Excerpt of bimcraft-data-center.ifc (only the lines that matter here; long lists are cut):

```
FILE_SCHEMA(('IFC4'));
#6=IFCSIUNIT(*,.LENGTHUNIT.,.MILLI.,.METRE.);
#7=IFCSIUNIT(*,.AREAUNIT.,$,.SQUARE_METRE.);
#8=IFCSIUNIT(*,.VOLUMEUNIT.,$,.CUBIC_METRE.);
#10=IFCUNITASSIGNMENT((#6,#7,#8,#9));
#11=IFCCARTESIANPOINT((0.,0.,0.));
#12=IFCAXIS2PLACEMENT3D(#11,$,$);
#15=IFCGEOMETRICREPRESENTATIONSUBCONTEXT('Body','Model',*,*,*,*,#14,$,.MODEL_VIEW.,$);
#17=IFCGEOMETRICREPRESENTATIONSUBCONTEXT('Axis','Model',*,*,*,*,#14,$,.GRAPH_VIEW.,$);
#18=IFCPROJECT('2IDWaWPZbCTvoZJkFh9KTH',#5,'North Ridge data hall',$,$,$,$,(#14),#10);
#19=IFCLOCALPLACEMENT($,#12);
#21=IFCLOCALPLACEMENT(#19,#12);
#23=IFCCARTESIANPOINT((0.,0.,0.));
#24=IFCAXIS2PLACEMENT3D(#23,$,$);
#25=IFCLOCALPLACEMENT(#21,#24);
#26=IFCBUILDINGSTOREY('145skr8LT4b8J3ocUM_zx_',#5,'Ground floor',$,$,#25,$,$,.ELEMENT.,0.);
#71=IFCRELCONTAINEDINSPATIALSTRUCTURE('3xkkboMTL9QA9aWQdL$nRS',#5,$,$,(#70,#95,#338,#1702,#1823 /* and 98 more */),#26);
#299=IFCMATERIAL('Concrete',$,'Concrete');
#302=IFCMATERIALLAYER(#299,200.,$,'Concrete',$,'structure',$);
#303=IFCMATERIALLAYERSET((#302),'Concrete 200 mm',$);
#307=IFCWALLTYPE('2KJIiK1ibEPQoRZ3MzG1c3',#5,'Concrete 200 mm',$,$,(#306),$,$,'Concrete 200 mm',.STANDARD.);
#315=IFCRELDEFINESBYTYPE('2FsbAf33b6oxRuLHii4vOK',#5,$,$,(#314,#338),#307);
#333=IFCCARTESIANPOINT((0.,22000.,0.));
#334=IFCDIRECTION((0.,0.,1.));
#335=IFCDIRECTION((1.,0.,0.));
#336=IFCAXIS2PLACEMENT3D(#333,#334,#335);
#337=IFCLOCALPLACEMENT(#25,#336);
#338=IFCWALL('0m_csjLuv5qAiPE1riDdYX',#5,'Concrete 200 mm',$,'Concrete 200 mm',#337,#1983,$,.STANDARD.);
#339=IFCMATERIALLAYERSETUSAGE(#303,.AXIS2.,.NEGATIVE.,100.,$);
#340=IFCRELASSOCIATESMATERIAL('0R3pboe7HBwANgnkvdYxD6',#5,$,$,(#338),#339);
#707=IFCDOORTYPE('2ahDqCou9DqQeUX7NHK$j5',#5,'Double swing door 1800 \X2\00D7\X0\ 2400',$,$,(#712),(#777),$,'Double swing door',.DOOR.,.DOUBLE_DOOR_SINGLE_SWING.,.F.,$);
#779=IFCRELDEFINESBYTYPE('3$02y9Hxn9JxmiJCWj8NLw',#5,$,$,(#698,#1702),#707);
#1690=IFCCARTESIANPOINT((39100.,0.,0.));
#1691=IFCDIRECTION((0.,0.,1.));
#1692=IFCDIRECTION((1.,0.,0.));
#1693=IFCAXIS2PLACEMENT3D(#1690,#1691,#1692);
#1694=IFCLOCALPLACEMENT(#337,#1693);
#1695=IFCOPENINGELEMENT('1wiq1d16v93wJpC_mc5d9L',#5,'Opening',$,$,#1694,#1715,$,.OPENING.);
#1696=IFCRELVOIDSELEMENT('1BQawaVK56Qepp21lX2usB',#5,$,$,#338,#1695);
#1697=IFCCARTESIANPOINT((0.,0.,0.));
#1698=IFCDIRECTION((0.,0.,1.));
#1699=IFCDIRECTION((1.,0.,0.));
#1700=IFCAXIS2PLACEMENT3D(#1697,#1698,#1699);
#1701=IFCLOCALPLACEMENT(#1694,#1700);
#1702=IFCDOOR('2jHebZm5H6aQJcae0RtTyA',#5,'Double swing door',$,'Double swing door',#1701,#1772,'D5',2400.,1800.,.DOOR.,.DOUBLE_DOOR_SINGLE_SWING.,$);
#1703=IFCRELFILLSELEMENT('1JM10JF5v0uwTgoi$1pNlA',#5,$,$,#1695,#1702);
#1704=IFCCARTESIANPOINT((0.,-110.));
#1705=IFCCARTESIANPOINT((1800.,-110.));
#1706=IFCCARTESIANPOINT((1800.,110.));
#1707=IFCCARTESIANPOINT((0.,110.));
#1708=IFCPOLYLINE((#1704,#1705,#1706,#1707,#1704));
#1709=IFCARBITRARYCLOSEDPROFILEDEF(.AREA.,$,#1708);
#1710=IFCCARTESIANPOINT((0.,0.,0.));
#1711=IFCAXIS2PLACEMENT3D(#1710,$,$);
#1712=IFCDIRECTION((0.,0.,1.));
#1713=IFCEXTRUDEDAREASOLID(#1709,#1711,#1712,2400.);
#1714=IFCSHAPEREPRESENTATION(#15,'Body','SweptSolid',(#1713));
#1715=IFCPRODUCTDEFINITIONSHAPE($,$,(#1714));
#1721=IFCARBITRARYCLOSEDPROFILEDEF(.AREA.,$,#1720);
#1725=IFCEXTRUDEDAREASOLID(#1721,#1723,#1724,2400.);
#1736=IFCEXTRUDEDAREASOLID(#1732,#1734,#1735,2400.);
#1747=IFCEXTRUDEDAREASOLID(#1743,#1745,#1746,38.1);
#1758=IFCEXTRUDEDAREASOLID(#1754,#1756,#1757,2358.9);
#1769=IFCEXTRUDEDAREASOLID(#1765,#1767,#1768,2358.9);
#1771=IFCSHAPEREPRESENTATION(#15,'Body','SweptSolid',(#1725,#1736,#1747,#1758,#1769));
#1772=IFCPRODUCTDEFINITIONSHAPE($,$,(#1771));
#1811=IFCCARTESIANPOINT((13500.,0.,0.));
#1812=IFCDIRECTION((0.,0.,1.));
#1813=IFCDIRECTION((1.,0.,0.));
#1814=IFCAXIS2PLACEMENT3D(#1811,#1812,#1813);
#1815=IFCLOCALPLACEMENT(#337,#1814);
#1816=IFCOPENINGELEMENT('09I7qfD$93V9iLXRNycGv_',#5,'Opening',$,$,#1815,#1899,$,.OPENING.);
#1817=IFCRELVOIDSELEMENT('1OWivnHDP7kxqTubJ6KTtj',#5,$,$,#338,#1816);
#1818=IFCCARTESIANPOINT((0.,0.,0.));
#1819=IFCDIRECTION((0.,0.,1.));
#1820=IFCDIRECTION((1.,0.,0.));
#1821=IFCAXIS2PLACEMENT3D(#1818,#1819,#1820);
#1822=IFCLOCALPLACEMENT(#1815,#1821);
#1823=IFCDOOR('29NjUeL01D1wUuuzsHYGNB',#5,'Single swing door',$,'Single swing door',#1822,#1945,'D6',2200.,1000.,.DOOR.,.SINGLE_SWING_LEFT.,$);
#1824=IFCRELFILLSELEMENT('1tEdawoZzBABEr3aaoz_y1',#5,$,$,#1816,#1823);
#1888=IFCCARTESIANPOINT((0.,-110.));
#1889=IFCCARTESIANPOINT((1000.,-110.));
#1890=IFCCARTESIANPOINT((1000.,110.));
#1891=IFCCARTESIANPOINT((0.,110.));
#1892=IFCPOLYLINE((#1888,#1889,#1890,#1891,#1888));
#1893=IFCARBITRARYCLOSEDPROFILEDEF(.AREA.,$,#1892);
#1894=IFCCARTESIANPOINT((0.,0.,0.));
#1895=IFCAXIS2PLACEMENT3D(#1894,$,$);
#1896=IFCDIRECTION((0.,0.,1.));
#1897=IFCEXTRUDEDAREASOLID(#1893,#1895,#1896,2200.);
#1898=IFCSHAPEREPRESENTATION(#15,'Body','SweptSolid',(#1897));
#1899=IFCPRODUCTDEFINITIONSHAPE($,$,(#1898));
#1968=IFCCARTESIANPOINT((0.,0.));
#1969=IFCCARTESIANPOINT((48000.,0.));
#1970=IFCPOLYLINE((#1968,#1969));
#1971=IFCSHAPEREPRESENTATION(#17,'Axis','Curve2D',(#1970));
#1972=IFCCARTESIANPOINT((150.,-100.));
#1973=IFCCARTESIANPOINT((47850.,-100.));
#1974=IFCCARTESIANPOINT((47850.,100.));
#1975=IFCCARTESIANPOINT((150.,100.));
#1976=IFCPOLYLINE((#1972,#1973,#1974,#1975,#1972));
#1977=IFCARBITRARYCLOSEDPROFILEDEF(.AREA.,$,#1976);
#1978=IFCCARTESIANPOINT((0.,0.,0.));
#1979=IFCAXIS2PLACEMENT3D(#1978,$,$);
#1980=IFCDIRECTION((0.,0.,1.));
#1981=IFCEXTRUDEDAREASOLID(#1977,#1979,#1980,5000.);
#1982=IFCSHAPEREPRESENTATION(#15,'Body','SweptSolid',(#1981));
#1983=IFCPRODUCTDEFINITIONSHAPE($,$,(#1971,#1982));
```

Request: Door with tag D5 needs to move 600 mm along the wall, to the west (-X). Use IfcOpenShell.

```python
import ifcopenshell
import ifcopenshell.api.geometry
import ifcopenshell.util.placement
import ifcopenshell.util.unit

model = ifcopenshell.open("bimcraft-data-center.ifc")
unit_scale = ifcopenshell.util.unit.calculate_unit_scale(model)

door = model.by_guid("2jHebZm5H6aQJcae0RtTyA")
opening = door.FillsVoids[0].RelatingOpeningElement
wall = opening.VoidsElements[0].RelatingBuildingElement

wall_matrix = ifcopenshell.util.placement.get_local_placement(wall.ObjectPlacement)
shift = wall_matrix[:3, 0] * -0.6 / unit_scale
before = ifcopenshell.util.placement.get_local_placement(door.ObjectPlacement)[:3, 3].copy()

# The door is placed relative to its opening, so it follows when the opening moves.
matrix = ifcopenshell.util.placement.get_local_placement(opening.ObjectPlacement)
matrix[:3, 3] += shift
ifcopenshell.api.geometry.edit_object_placement(
    model, product=opening, matrix=matrix, is_si=False, should_transform_children=True
)

after = ifcopenshell.util.placement.get_local_placement(door.ObjectPlacement)[:3, 3]
print("door moved by", (after - before).round(3) + 0.0)

model.write("bimcraft-data-center_edited.ifc")
```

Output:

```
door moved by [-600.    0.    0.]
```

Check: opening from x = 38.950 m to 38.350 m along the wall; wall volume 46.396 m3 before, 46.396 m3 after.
